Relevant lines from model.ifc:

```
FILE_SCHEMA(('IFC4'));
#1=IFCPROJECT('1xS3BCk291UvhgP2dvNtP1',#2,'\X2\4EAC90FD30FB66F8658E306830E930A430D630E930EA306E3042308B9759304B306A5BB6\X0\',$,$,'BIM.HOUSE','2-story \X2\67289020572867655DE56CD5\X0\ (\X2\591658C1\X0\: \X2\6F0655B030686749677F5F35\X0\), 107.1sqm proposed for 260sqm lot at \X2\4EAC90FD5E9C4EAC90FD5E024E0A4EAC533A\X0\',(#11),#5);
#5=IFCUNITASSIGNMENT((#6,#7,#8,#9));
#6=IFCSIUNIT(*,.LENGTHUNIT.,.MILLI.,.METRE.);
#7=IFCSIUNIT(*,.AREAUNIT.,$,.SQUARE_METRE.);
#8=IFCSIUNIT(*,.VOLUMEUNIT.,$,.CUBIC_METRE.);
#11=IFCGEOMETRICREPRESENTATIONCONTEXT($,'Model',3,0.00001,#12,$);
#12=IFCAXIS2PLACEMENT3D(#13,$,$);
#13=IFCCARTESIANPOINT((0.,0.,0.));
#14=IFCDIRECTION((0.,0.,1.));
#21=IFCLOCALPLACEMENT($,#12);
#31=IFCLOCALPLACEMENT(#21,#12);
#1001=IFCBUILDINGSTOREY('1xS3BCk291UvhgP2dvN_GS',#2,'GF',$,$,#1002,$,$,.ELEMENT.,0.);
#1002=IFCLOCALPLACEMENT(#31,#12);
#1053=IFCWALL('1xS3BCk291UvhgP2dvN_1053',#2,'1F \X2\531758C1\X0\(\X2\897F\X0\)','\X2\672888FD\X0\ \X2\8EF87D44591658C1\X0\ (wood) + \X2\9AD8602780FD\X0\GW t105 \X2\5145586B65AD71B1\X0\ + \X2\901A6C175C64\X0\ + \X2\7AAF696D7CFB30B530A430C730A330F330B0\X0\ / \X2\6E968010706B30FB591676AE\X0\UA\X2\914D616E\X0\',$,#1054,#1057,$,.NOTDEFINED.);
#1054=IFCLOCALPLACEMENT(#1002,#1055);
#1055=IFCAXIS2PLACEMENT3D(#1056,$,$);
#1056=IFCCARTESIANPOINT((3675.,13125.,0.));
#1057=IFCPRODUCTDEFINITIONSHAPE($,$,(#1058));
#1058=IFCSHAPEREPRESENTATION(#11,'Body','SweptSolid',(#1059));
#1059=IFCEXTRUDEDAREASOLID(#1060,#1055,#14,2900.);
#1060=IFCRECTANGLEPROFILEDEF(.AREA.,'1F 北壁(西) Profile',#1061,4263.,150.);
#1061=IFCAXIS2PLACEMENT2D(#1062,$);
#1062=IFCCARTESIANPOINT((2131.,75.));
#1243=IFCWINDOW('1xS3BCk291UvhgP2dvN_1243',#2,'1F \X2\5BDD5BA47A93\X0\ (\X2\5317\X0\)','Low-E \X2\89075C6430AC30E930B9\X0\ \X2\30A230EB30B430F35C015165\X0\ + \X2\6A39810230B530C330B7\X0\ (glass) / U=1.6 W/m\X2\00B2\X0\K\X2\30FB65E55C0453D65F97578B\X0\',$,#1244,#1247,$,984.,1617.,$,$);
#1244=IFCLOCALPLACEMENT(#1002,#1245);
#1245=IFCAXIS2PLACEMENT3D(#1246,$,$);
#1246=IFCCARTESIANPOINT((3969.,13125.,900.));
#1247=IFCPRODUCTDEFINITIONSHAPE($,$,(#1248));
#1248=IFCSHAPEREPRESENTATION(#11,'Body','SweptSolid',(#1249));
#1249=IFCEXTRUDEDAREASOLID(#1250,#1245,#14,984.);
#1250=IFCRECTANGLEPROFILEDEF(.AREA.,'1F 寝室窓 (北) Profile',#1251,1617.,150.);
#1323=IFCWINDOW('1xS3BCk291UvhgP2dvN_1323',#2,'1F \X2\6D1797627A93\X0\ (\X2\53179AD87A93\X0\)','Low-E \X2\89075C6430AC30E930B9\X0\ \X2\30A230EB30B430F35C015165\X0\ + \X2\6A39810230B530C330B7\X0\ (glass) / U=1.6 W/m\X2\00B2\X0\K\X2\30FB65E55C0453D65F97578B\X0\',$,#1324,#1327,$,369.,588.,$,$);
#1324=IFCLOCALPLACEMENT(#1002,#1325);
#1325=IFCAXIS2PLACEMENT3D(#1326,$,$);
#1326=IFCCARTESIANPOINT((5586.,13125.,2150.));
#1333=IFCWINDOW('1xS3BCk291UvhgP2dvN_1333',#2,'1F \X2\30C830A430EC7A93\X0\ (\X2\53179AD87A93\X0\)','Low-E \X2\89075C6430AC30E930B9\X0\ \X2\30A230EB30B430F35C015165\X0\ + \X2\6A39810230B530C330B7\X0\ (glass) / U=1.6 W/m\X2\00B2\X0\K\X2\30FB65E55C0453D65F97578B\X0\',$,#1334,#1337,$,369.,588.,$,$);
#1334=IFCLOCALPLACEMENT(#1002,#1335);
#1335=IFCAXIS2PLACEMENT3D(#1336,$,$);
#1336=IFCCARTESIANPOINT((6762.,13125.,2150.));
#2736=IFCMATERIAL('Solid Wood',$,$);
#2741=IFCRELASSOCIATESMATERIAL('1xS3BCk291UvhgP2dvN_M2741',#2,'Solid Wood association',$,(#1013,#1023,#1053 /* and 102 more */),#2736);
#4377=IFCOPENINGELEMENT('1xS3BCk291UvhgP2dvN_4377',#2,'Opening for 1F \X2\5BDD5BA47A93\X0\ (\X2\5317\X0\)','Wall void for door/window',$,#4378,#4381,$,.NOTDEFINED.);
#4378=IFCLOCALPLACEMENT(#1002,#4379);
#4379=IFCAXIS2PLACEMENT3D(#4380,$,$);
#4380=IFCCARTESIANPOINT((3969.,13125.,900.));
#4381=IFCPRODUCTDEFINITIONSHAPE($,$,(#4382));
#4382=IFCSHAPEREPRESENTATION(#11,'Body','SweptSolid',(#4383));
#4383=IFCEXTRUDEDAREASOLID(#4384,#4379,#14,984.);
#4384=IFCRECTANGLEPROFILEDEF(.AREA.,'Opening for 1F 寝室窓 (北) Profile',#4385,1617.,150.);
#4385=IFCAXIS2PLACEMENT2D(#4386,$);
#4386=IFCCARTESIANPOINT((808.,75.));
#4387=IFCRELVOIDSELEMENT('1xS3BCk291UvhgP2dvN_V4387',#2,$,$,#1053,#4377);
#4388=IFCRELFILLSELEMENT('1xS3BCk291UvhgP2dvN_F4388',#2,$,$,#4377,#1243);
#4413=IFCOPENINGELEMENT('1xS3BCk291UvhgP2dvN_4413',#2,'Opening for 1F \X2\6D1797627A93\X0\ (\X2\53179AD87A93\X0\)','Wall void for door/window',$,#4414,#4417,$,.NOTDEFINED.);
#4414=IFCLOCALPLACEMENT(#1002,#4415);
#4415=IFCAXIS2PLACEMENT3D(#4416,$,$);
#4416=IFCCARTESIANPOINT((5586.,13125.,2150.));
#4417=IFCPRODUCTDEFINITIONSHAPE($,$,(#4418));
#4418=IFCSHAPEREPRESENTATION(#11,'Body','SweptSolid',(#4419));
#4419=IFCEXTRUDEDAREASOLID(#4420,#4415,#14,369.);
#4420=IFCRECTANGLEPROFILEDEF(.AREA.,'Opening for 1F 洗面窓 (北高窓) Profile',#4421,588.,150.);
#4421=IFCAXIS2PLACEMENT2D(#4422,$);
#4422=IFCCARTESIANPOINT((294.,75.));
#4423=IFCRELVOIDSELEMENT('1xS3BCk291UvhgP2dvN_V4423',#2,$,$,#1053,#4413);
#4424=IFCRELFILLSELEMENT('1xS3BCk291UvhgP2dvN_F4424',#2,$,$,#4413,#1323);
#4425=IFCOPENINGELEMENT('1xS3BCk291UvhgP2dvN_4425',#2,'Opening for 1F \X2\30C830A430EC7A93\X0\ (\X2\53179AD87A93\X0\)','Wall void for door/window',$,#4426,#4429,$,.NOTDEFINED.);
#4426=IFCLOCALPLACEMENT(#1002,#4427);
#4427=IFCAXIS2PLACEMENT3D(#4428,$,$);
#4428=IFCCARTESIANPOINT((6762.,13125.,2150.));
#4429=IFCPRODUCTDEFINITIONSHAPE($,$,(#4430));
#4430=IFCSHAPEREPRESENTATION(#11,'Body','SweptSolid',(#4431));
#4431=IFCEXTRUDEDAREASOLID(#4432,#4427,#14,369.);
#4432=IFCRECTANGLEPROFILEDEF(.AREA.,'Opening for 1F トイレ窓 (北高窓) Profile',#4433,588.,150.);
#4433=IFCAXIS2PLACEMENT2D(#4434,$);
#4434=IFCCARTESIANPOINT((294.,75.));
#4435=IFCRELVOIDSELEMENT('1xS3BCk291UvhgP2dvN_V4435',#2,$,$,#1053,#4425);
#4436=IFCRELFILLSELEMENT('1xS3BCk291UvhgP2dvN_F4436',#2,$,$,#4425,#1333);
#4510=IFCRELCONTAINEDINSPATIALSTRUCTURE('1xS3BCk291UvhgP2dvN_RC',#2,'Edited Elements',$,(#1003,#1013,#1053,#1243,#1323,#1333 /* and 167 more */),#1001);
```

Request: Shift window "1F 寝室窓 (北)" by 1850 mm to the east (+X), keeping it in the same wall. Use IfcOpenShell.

```python
import ifcopenshell
import ifcopenshell.api.geometry
import ifcopenshell.util.placement
import ifcopenshell.util.unit

model = ifcopenshell.open("model.ifc")
unit_scale = ifcopenshell.util.unit.calculate_unit_scale(model)

window = model.by_guid("1xS3BCk291UvhgP2dvN_1243")
opening = window.FillsVoids[0].RelatingOpeningElement
wall = opening.VoidsElements[0].RelatingBuildingElement

wall_matrix = ifcopenshell.util.placement.get_local_placement(wall.ObjectPlacement)
shift = wall_matrix[:3, 0] * 1.85 / unit_scale
before = ifcopenshell.util.placement.get_local_placement(window.ObjectPlacement)[:3, 3].copy()

# The window is not placed relative to its opening, so move both.
for product in (opening, window):
    matrix = ifcopenshell.util.placement.get_local_placement(product.ObjectPlacement)
    matrix[:3, 3] += shift
    ifcopenshell.api.geometry.edit_object_placement(model, product=product, matrix=matrix, is_si=False)

after = ifcopenshell.util.placement.get_local_placement(window.ObjectPlacement)[:3, 3]
print("window moved by", (after - before).round(3) + 0.0)

model.write("model_edited.ifc")
```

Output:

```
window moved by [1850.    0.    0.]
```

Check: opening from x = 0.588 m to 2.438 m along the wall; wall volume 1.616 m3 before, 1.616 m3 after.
